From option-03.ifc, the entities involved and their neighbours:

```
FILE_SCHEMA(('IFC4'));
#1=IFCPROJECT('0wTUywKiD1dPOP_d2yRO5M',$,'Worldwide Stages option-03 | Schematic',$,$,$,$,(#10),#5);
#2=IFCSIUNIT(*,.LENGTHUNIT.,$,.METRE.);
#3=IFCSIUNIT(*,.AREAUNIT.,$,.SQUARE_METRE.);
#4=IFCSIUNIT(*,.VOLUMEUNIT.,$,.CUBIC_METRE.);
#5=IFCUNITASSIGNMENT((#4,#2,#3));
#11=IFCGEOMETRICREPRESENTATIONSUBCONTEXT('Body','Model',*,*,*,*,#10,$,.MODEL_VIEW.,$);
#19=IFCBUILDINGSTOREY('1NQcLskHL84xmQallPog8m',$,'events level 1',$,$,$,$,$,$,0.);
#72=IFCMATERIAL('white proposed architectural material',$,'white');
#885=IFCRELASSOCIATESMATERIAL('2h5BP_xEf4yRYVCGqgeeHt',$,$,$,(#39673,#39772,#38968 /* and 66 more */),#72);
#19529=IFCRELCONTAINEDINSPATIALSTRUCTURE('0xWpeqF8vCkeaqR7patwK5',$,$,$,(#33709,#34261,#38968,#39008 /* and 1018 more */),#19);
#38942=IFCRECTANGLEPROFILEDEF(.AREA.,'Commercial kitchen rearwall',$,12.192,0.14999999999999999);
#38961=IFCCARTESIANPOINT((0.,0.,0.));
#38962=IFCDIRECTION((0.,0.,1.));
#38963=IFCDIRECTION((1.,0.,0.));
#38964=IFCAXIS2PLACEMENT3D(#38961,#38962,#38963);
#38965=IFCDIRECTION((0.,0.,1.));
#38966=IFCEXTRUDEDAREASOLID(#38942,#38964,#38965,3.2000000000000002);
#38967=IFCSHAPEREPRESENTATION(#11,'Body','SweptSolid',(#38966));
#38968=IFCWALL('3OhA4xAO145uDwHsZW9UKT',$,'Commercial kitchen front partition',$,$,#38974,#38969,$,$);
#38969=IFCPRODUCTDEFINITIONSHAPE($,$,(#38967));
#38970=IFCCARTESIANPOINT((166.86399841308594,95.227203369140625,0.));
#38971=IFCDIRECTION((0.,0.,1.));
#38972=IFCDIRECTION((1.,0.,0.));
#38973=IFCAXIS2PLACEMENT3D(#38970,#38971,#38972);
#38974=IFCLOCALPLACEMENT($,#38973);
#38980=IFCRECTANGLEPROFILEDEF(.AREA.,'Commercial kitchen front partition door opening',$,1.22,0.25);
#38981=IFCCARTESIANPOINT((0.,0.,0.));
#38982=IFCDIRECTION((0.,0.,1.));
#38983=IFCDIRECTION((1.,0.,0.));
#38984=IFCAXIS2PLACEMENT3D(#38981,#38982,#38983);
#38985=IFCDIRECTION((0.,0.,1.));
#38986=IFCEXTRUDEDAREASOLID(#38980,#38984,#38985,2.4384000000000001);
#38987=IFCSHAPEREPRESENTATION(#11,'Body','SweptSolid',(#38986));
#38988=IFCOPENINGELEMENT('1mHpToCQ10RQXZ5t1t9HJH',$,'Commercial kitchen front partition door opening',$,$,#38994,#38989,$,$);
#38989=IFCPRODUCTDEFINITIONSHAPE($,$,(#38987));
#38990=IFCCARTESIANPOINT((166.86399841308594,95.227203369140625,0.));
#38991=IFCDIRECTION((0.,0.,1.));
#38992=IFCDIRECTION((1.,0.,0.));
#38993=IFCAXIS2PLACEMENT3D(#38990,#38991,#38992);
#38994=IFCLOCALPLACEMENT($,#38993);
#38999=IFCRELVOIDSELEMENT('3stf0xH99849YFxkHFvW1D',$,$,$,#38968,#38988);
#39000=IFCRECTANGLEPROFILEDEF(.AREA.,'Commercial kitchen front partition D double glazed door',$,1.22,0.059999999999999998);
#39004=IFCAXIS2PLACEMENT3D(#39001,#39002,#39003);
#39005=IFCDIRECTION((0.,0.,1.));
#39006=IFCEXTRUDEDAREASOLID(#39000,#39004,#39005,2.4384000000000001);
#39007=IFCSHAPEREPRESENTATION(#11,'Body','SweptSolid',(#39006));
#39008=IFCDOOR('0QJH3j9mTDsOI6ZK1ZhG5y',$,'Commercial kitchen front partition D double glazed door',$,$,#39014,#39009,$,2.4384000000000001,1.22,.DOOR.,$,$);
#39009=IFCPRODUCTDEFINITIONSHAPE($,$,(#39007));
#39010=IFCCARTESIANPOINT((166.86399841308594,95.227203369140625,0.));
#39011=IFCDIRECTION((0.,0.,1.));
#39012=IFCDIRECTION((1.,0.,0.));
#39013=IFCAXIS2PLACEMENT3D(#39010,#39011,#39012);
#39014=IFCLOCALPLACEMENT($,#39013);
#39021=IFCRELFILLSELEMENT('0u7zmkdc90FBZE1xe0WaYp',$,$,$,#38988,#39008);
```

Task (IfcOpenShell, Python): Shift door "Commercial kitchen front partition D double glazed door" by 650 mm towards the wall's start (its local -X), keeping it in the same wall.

```python
import ifcopenshell
import ifcopenshell.api.geometry
import ifcopenshell.util.placement
import ifcopenshell.util.unit

model = ifcopenshell.open("option-03.ifc")
unit_scale = ifcopenshell.util.unit.calculate_unit_scale(model)

door = model.by_guid("0QJH3j9mTDsOI6ZK1ZhG5y")
opening = door.FillsVoids[0].RelatingOpeningElement
wall = opening.VoidsElements[0].RelatingBuildingElement

wall_matrix = ifcopenshell.util.placement.get_local_placement(wall.ObjectPlacement)
shift = wall_matrix[:3, 0] * -0.65 / unit_scale
before = ifcopenshell.util.placement.get_local_placement(door.ObjectPlacement)[:3, 3].copy()

# The door is not placed relative to its opening, so move both.
for product in (opening, door):
    matrix = ifcopenshell.util.placement.get_local_placement(product.ObjectPlacement)
    matrix[:3, 3] += shift
    ifcopenshell.api.geometry.edit_object_placement(model, product=product, matrix=matrix, is_si=False)

after = ifcopenshell.util.placement.get_local_placement(door.ObjectPlacement)[:3, 3]
print("door moved by", (after - before).round(3) + 0.0)

model.write("option-03_updated.ifc")
```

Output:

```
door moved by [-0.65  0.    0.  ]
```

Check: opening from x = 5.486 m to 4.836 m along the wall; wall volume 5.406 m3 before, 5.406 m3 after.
